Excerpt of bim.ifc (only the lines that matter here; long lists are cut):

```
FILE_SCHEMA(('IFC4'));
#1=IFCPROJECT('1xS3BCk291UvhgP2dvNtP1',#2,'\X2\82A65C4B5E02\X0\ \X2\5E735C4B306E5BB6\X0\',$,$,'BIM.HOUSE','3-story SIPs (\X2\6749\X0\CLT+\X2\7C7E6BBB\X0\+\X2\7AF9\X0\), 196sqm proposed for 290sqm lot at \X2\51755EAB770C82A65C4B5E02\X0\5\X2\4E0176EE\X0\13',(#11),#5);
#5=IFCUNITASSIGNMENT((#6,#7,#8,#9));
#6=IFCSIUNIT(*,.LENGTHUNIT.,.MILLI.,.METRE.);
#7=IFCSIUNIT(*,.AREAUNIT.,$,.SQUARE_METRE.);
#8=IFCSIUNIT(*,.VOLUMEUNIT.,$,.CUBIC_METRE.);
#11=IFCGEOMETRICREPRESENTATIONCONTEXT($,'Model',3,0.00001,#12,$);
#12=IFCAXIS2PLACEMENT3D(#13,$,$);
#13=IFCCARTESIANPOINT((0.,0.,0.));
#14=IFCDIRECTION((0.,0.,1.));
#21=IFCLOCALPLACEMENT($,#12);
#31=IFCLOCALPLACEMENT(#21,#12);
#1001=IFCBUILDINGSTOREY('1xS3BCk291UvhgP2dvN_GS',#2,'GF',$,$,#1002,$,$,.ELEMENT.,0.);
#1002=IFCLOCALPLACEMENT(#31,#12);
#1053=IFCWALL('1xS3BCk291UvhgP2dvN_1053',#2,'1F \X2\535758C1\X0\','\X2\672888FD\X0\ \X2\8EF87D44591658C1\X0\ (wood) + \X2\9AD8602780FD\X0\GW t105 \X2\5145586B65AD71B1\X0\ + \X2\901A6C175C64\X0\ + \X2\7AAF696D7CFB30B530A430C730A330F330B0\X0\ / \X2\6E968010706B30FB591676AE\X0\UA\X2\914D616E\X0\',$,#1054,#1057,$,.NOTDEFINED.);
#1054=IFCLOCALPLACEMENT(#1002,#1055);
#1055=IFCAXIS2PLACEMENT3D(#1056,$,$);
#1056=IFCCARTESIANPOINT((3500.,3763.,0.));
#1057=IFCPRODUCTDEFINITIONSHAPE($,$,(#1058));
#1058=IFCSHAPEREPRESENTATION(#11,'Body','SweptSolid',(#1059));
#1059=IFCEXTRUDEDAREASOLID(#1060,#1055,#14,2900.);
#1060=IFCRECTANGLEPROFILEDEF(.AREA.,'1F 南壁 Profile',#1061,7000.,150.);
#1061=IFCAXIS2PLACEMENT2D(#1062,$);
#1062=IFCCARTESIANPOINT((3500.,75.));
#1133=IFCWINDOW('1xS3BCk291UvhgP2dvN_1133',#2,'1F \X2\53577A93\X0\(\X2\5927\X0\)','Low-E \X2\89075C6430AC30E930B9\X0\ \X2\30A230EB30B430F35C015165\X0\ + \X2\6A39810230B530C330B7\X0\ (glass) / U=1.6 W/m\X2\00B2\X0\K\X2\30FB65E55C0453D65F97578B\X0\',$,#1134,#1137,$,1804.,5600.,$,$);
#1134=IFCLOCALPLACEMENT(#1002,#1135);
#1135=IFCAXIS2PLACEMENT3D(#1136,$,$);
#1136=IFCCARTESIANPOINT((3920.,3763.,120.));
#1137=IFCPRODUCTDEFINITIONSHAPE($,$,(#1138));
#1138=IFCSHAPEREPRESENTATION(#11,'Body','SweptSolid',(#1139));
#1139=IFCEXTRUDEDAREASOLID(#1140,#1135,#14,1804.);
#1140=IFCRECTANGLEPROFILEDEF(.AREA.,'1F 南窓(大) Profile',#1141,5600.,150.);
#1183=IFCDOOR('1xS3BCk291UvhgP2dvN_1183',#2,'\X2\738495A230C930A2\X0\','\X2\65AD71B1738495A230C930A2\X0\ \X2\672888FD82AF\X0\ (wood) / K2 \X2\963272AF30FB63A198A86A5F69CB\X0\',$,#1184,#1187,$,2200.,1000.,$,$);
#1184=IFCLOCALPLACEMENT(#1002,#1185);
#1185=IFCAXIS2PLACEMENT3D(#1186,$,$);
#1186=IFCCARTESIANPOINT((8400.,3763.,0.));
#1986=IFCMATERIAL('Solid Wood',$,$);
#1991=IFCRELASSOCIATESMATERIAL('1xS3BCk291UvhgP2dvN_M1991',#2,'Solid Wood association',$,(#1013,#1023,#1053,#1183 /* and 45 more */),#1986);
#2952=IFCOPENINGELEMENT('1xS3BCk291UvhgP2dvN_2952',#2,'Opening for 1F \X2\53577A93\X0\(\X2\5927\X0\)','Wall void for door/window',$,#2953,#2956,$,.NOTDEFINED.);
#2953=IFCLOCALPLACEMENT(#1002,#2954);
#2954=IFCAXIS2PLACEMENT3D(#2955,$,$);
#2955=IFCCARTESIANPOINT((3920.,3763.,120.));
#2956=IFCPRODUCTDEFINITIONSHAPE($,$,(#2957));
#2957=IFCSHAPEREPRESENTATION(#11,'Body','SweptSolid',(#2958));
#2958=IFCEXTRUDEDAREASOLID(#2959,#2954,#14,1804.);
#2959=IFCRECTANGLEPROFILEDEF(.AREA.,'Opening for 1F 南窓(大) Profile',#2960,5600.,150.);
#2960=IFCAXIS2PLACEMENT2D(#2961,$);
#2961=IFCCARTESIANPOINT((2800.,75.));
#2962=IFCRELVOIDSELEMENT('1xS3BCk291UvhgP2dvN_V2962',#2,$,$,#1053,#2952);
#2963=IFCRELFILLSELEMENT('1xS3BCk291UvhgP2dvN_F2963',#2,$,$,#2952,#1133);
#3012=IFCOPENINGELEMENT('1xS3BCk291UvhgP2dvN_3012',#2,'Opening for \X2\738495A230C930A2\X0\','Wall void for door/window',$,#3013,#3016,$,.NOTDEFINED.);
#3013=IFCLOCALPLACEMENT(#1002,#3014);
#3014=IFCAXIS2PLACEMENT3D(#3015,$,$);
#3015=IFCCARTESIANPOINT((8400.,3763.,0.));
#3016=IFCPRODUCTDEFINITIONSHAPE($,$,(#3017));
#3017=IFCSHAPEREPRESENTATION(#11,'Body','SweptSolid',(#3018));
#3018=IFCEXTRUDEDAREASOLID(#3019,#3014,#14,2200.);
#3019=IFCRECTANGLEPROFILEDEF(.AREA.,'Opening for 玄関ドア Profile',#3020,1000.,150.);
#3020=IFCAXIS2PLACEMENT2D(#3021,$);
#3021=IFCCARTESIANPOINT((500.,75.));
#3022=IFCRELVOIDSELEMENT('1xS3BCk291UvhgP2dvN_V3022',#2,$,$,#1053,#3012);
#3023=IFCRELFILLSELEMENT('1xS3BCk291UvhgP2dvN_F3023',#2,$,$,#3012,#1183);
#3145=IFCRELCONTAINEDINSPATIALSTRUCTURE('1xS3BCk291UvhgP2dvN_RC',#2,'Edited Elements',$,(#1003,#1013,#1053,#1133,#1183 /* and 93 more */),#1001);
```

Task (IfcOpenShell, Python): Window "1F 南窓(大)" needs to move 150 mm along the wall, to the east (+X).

```python
import ifcopenshell
import ifcopenshell.api.geometry
import ifcopenshell.util.placement
import ifcopenshell.util.unit

model = ifcopenshell.open("bim.ifc")
unit_scale = ifcopenshell.util.unit.calculate_unit_scale(model)

window = model.by_guid("1xS3BCk291UvhgP2dvN_1133")
opening = window.FillsVoids[0].RelatingOpeningElement
wall = opening.VoidsElements[0].RelatingBuildingElement

wall_matrix = ifcopenshell.util.placement.get_local_placement(wall.ObjectPlacement)
shift = wall_matrix[:3, 0] * 0.15 / unit_scale
before = ifcopenshell.util.placement.get_local_placement(window.ObjectPlacement)[:3, 3].copy()

# The window is not placed relative to its opening, so move both.
for product in (opening, window):
    matrix = ifcopenshell.util.placement.get_local_placement(product.ObjectPlacement)
    matrix[:3, 3] += shift
    ifcopenshell.api.geometry.edit_object_placement(model, product=product, matrix=matrix, is_si=False)

after = ifcopenshell.util.placement.get_local_placement(window.ObjectPlacement)[:3, 3]
print("window moved by", (after - before).round(3) + 0.0)

model.write("bim_rev.ifc")
```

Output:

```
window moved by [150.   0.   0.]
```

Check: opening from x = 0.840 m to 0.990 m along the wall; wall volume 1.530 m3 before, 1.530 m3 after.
